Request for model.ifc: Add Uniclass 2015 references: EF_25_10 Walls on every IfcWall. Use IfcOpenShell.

First a look at what the model holds.

```python
import ifcopenshell

model = ifcopenshell.open("model.ifc")
print(model.schema)
print("classifications:", [c.Name for c in model.by_type("IfcClassification")])
for ifc_class in ("IfcDoor", "IfcRoof", "IfcStair", "IfcWall", "IfcWindow"):
    print(ifc_class, len(model.by_type(ifc_class)))
```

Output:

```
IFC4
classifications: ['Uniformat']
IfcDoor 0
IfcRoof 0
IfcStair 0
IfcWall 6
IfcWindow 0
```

```python
import ifcopenshell
import ifcopenshell.api.classification

model = ifcopenshell.open("model.ifc")

system = ifcopenshell.api.classification.add_classification(model, classification="Uniclass 2015")

codes = {
    "IfcWall": ("EF_25_10", "Walls"),
}
for ifc_class, (code, name) in codes.items():
    products = model.by_type(ifc_class)
    ifcopenshell.api.classification.add_reference(
        model, products=products, classification=system, identification=code, name=name
    )
    print(code, len(products))

model.write("model_edited.ifc")
```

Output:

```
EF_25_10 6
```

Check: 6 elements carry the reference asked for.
